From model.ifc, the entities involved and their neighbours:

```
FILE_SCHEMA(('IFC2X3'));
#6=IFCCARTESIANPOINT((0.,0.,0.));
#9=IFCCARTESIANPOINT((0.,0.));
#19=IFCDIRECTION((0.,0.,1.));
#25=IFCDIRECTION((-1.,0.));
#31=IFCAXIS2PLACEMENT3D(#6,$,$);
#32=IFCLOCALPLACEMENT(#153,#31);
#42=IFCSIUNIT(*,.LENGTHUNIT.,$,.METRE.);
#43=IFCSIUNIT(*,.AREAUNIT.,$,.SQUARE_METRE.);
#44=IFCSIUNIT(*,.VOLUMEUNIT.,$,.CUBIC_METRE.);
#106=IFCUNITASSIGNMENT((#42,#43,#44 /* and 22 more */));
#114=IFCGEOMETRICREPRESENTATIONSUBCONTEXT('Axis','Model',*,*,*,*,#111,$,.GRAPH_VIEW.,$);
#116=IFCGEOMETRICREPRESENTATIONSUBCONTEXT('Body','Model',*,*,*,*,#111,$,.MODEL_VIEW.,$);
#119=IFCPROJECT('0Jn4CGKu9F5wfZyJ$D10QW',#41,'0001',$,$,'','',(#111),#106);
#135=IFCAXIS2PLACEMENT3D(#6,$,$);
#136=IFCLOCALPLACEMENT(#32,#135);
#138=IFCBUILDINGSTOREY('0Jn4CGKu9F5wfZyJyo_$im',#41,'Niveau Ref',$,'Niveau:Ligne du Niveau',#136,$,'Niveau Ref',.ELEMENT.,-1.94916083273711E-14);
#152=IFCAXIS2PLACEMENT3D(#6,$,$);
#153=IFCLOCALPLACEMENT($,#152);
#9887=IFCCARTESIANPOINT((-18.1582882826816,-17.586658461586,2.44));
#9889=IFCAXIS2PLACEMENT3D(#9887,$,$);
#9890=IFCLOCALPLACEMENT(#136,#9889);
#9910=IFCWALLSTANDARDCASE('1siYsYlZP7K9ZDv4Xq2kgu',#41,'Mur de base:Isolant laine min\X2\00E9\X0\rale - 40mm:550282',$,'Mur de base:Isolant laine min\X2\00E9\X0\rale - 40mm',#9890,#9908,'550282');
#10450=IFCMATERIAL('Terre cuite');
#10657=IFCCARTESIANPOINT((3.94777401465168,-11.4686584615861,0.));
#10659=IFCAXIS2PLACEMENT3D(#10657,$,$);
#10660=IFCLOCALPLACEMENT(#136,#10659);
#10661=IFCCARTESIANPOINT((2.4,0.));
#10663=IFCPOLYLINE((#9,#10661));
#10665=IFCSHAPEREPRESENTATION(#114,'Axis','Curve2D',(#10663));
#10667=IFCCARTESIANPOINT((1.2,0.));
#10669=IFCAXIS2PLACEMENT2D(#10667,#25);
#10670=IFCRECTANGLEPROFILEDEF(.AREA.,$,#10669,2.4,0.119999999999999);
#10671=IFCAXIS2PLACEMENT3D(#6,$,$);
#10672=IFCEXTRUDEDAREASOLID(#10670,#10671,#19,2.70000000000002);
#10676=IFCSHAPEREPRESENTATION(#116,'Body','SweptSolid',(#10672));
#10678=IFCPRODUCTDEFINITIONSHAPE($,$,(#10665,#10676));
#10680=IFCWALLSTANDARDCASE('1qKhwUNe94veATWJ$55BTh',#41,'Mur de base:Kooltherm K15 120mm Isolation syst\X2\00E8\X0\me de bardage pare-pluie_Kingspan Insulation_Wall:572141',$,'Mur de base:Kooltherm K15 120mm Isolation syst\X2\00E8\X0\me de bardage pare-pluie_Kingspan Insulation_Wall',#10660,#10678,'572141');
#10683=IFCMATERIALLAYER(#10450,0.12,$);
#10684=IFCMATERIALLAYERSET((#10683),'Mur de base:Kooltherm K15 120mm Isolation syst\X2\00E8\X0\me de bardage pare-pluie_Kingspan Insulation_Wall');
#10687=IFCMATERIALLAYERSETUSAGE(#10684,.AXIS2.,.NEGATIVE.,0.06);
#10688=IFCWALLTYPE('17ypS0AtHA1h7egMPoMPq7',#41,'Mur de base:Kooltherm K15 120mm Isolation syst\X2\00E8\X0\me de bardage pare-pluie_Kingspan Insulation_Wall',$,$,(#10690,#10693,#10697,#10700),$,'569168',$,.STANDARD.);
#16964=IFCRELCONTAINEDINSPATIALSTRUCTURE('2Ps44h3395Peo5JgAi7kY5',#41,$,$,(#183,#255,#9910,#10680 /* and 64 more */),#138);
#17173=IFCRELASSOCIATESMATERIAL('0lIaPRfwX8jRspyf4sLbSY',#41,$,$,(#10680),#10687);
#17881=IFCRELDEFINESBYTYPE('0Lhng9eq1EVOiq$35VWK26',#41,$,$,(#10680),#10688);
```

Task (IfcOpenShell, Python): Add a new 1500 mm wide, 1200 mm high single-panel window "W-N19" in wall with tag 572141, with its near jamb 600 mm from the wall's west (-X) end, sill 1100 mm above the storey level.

```python
import numpy as np
import ifcopenshell
import ifcopenshell.api.feature
import ifcopenshell.api.geometry
import ifcopenshell.api.root
import ifcopenshell.api.spatial
import ifcopenshell.api.type
import ifcopenshell.geom
import ifcopenshell.util.element
import ifcopenshell.util.placement
import ifcopenshell.util.representation
import ifcopenshell.util.shape
import ifcopenshell.util.unit

model = ifcopenshell.open("model.ifc")
unit_scale = ifcopenshell.util.unit.calculate_unit_scale(model)
settings = ifcopenshell.geom.settings()


def volume(element):
    """Net volume in cubic metres, openings subtracted."""
    shape = ifcopenshell.geom.create_shape(settings, element)
    return ifcopenshell.util.shape.get_volume(shape.geometry)


wall = model.by_id(10680)
storey = ifcopenshell.util.element.get_container(wall, ifc_class="IfcBuildingStorey")
context = ifcopenshell.util.representation.get_context(model, "Model", "Body", "MODEL_VIEW")
before = volume(wall)

width, height, from_end, sill = 1.5, 1.2, 0.6, 1.1  # metres

# The wall runs along its own X axis, and the end named is its -X end.
wall_shape = ifcopenshell.geom.create_shape(settings, wall)
x, y, z = ifcopenshell.util.shape.get_vertices(wall_shape.geometry).T
start = x.min() + from_end
face, thickness = float(y.min()), float(y.max() - y.min())
wall_matrix = ifcopenshell.util.placement.get_local_placement(wall.ObjectPlacement)
level = ifcopenshell.util.placement.get_local_placement(storey.ObjectPlacement)[2, 3]


def in_wall(x, y):
    """Placement at x, y metres in the wall's axes, at sill height."""
    matrix = wall_matrix.copy()
    matrix[:, 3] = wall_matrix @ np.array([x / unit_scale, y / unit_scale, 0.0, 1.0])
    matrix[2, 3] = level + sill / unit_scale
    return matrix


# Opening: a box that overshoots both wall faces by 50 mm.
opening = ifcopenshell.api.root.create_entity(model, ifc_class="IfcOpeningElement")
box = ifcopenshell.api.geometry.add_wall_representation(
    model, context=context, length=width, height=height, thickness=thickness + 0.1
)
ifcopenshell.api.geometry.assign_representation(model, product=opening, representation=box)
ifcopenshell.api.geometry.edit_object_placement(model, product=opening, matrix=in_wall(start, face - 0.05), is_si=False)
ifcopenshell.api.feature.add_feature(model, feature=opening, element=wall)

window = ifcopenshell.api.root.create_entity(model, ifc_class="IfcWindow", name="W-N19")
window.OverallWidth, window.OverallHeight = width / unit_scale, height / unit_scale
body = ifcopenshell.api.geometry.add_window_representation(
    model,
    context=context,
    overall_width=window.OverallWidth,
    overall_height=window.OverallHeight,
    partition_type="SINGLE_PANEL",
)
ifcopenshell.api.geometry.assign_representation(model, product=window, representation=body)
ifcopenshell.api.spatial.assign_container(model, products=[window], relating_structure=storey)
fills = ifcopenshell.api.feature.add_filling(model, opening=opening, element=window)
fills.OwnerHistory = window.OwnerHistory  # required in IFC2X3

# IFC2X3 keeps the operation on the window style.
style = ifcopenshell.api.root.create_entity(model, ifc_class="IfcWindowStyle", name="W-N19")
style.OperationType, style.ConstructionType = "SINGLE_PANEL", "NOTDEFINED"
style.ParameterTakesPrecedence = style.Sizeable = False
ifcopenshell.api.type.assign_type(model, related_objects=[window], relating_type=style)

# Centre the window in the wall's thickness.
ifcopenshell.api.geometry.edit_object_placement(model, product=window, matrix=in_wall(start, face), is_si=False)
window_shape = ifcopenshell.geom.create_shape(settings, window)
depth = ifcopenshell.util.shape.get_vertices(window_shape.geometry)[:, 1]
offset = face + thickness / 2 - (depth.min() + depth.max()) / 2
ifcopenshell.api.geometry.edit_object_placement(model, product=window, matrix=in_wall(start, offset), is_si=False)

after = volume(wall)

print(f"wall volume {before:.3f} -> {after:.3f} m3")

model.write("model_edited.ifc")
```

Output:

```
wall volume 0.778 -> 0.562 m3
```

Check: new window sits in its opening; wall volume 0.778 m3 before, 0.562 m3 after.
